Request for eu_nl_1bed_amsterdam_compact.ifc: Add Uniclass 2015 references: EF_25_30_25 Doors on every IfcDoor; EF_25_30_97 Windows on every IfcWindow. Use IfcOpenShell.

First a look at what the model holds.

```python
import ifcopenshell

model = ifcopenshell.open("eu_nl_1bed_amsterdam_compact.ifc")
print(model.schema)
print("classifications:", [c.Name for c in model.by_type("IfcClassification")])
for ifc_class in ("IfcDoor", "IfcRoof", "IfcStair", "IfcWall", "IfcWindow"):
    print(ifc_class, len(model.by_type(ifc_class)))
```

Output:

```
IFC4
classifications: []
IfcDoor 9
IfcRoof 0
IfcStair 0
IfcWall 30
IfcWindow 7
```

```python
import ifcopenshell
import ifcopenshell.api.classification

model = ifcopenshell.open("eu_nl_1bed_amsterdam_compact.ifc")

system = ifcopenshell.api.classification.add_classification(model, classification="Uniclass 2015")

codes = {
    "IfcDoor": ("EF_25_30_25", "Doors"),
    "IfcWindow": ("EF_25_30_97", "Windows"),
}
for ifc_class, (code, name) in codes.items():
    products = model.by_type(ifc_class)
    ifcopenshell.api.classification.add_reference(
        model, products=products, classification=system, identification=code, name=name
    )
    print(code, len(products))

model.write("eu_nl_1bed_amsterdam_compact-out.ifc")
```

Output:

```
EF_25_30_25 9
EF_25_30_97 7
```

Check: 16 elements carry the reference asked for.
